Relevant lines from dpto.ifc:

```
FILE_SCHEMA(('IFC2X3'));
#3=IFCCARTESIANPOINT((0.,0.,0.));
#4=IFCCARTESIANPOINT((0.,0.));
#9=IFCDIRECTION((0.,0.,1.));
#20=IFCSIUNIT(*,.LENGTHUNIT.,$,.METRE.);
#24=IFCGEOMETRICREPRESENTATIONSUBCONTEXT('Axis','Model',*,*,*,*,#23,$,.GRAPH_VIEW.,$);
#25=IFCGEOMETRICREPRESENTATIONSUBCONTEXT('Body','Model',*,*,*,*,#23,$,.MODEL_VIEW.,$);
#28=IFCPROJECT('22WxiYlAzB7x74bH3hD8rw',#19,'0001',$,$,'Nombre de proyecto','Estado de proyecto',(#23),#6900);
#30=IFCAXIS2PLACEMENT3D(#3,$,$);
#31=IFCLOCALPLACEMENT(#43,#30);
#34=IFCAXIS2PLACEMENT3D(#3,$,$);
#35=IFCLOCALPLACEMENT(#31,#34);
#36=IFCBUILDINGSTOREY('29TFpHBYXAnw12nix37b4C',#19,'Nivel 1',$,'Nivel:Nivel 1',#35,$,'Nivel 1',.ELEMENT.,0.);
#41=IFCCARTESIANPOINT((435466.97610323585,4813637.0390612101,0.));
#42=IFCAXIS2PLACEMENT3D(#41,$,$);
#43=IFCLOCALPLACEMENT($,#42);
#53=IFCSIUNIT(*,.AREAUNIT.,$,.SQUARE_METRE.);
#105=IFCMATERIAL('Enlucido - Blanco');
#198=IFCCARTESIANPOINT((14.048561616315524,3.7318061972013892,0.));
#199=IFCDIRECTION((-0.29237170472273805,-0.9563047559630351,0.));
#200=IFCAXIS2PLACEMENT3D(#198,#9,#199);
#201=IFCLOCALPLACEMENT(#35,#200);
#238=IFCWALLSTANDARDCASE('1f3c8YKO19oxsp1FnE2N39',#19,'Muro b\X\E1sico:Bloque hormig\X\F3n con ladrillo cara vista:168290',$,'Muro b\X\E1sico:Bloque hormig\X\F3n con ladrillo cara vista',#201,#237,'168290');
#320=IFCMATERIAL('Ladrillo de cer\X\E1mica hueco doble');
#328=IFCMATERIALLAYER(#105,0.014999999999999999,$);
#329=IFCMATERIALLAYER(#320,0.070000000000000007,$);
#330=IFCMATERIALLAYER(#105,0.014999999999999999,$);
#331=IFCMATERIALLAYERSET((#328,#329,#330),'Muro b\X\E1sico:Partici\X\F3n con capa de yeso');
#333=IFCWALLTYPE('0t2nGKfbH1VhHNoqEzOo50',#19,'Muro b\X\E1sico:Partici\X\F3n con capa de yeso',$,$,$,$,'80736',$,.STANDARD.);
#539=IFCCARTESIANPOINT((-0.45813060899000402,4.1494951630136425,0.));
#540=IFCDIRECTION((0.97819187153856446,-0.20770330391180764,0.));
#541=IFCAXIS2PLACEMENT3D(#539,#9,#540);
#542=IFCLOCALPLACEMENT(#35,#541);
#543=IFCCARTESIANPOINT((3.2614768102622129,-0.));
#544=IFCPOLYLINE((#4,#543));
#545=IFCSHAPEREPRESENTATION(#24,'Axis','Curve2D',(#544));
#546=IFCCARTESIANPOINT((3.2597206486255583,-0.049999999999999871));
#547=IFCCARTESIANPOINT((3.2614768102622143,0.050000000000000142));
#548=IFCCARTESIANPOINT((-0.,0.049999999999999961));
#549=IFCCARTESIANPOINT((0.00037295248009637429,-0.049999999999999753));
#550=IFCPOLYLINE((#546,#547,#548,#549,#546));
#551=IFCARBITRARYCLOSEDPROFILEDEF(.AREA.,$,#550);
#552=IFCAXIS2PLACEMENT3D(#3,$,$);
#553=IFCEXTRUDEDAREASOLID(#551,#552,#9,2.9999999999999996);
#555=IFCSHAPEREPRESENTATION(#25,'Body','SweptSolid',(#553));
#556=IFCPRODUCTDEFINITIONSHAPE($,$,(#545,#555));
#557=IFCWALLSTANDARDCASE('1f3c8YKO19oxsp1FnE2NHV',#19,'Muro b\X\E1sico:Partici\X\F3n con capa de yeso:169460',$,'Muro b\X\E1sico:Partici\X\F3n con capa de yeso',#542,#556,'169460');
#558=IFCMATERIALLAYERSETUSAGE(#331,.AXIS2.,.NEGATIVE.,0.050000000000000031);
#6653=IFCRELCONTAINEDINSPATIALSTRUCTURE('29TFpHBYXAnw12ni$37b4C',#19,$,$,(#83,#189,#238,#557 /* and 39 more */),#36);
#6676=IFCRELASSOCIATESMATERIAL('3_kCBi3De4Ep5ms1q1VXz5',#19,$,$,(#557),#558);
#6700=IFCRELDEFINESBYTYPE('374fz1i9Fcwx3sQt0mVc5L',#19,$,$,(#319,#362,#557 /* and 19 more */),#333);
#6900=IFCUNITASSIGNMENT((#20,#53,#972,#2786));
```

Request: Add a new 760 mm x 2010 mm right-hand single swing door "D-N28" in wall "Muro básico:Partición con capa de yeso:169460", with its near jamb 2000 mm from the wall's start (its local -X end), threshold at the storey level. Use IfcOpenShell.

```python
import numpy as np
import ifcopenshell
import ifcopenshell.api.feature
import ifcopenshell.api.geometry
import ifcopenshell.api.root
import ifcopenshell.api.spatial
import ifcopenshell.api.type
import ifcopenshell.geom
import ifcopenshell.util.element
import ifcopenshell.util.placement
import ifcopenshell.util.representation
import ifcopenshell.util.shape
import ifcopenshell.util.unit

model = ifcopenshell.open("dpto.ifc")
unit_scale = ifcopenshell.util.unit.calculate_unit_scale(model)
settings = ifcopenshell.geom.settings()


def volume(element):
    """Net volume in cubic metres, openings subtracted."""
    shape = ifcopenshell.geom.create_shape(settings, element)
    return ifcopenshell.util.shape.get_volume(shape.geometry)


wall = model.by_id(557)
storey = ifcopenshell.util.element.get_container(wall, ifc_class="IfcBuildingStorey")
context = ifcopenshell.util.representation.get_context(model, "Model", "Body", "MODEL_VIEW")
before = volume(wall)

width, height, from_end, sill = 0.76, 2.01, 2, 0.0  # metres

# The wall runs along its own X axis, and the end named is its -X end.
wall_shape = ifcopenshell.geom.create_shape(settings, wall)
x, y, z = ifcopenshell.util.shape.get_vertices(wall_shape.geometry).T
start = x.min() + from_end
face, thickness = float(y.min()), float(y.max() - y.min())
wall_matrix = ifcopenshell.util.placement.get_local_placement(wall.ObjectPlacement)
level = ifcopenshell.util.placement.get_local_placement(storey.ObjectPlacement)[2, 3]


def in_wall(x, y):
    """Placement at x, y metres in the wall's axes, at sill height."""
    matrix = wall_matrix.copy()
    matrix[:, 3] = wall_matrix @ np.array([x / unit_scale, y / unit_scale, 0.0, 1.0])
    matrix[2, 3] = level + sill / unit_scale
    return matrix


# Opening: a box that overshoots both wall faces by 50 mm.
opening = ifcopenshell.api.root.create_entity(model, ifc_class="IfcOpeningElement")
box = ifcopenshell.api.geometry.add_wall_representation(
    model, context=context, length=width, height=height, thickness=thickness + 0.1
)
ifcopenshell.api.geometry.assign_representation(model, product=opening, representation=box)
ifcopenshell.api.geometry.edit_object_placement(model, product=opening, matrix=in_wall(start, face - 0.05), is_si=False)
ifcopenshell.api.feature.add_feature(model, feature=opening, element=wall)

door = ifcopenshell.api.root.create_entity(model, ifc_class="IfcDoor", name="D-N28")
door.OverallWidth, door.OverallHeight = width / unit_scale, height / unit_scale
body = ifcopenshell.api.geometry.add_door_representation(
    model,
    context=context,
    overall_width=door.OverallWidth,
    overall_height=door.OverallHeight,
    operation_type="SINGLE_SWING_RIGHT",
    lining_properties={"LiningDepth": thickness / unit_scale, "ThresholdDepth": thickness / unit_scale},
)
ifcopenshell.api.geometry.assign_representation(model, product=door, representation=body)
ifcopenshell.api.spatial.assign_container(model, products=[door], relating_structure=storey)
fills = ifcopenshell.api.feature.add_filling(model, opening=opening, element=door)
fills.OwnerHistory = door.OwnerHistory  # required in IFC2X3

# IFC2X3 keeps the operation on the door style.
style = ifcopenshell.api.root.create_entity(model, ifc_class="IfcDoorStyle", name="D-N28")
style.OperationType, style.ConstructionType = "SINGLE_SWING_RIGHT", "NOTDEFINED"
style.ParameterTakesPrecedence = style.Sizeable = False
ifcopenshell.api.type.assign_type(model, related_objects=[door], relating_type=style)

# The lining spans the wall, so the door starts at the wall face.
ifcopenshell.api.geometry.edit_object_placement(model, product=door, matrix=in_wall(start, face), is_si=False)

after = volume(wall)

print(f"wall volume {before:.3f} -> {after:.3f} m3")

model.write("dpto_rev.ifc")
```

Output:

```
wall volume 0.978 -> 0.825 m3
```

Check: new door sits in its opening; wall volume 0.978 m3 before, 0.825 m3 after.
